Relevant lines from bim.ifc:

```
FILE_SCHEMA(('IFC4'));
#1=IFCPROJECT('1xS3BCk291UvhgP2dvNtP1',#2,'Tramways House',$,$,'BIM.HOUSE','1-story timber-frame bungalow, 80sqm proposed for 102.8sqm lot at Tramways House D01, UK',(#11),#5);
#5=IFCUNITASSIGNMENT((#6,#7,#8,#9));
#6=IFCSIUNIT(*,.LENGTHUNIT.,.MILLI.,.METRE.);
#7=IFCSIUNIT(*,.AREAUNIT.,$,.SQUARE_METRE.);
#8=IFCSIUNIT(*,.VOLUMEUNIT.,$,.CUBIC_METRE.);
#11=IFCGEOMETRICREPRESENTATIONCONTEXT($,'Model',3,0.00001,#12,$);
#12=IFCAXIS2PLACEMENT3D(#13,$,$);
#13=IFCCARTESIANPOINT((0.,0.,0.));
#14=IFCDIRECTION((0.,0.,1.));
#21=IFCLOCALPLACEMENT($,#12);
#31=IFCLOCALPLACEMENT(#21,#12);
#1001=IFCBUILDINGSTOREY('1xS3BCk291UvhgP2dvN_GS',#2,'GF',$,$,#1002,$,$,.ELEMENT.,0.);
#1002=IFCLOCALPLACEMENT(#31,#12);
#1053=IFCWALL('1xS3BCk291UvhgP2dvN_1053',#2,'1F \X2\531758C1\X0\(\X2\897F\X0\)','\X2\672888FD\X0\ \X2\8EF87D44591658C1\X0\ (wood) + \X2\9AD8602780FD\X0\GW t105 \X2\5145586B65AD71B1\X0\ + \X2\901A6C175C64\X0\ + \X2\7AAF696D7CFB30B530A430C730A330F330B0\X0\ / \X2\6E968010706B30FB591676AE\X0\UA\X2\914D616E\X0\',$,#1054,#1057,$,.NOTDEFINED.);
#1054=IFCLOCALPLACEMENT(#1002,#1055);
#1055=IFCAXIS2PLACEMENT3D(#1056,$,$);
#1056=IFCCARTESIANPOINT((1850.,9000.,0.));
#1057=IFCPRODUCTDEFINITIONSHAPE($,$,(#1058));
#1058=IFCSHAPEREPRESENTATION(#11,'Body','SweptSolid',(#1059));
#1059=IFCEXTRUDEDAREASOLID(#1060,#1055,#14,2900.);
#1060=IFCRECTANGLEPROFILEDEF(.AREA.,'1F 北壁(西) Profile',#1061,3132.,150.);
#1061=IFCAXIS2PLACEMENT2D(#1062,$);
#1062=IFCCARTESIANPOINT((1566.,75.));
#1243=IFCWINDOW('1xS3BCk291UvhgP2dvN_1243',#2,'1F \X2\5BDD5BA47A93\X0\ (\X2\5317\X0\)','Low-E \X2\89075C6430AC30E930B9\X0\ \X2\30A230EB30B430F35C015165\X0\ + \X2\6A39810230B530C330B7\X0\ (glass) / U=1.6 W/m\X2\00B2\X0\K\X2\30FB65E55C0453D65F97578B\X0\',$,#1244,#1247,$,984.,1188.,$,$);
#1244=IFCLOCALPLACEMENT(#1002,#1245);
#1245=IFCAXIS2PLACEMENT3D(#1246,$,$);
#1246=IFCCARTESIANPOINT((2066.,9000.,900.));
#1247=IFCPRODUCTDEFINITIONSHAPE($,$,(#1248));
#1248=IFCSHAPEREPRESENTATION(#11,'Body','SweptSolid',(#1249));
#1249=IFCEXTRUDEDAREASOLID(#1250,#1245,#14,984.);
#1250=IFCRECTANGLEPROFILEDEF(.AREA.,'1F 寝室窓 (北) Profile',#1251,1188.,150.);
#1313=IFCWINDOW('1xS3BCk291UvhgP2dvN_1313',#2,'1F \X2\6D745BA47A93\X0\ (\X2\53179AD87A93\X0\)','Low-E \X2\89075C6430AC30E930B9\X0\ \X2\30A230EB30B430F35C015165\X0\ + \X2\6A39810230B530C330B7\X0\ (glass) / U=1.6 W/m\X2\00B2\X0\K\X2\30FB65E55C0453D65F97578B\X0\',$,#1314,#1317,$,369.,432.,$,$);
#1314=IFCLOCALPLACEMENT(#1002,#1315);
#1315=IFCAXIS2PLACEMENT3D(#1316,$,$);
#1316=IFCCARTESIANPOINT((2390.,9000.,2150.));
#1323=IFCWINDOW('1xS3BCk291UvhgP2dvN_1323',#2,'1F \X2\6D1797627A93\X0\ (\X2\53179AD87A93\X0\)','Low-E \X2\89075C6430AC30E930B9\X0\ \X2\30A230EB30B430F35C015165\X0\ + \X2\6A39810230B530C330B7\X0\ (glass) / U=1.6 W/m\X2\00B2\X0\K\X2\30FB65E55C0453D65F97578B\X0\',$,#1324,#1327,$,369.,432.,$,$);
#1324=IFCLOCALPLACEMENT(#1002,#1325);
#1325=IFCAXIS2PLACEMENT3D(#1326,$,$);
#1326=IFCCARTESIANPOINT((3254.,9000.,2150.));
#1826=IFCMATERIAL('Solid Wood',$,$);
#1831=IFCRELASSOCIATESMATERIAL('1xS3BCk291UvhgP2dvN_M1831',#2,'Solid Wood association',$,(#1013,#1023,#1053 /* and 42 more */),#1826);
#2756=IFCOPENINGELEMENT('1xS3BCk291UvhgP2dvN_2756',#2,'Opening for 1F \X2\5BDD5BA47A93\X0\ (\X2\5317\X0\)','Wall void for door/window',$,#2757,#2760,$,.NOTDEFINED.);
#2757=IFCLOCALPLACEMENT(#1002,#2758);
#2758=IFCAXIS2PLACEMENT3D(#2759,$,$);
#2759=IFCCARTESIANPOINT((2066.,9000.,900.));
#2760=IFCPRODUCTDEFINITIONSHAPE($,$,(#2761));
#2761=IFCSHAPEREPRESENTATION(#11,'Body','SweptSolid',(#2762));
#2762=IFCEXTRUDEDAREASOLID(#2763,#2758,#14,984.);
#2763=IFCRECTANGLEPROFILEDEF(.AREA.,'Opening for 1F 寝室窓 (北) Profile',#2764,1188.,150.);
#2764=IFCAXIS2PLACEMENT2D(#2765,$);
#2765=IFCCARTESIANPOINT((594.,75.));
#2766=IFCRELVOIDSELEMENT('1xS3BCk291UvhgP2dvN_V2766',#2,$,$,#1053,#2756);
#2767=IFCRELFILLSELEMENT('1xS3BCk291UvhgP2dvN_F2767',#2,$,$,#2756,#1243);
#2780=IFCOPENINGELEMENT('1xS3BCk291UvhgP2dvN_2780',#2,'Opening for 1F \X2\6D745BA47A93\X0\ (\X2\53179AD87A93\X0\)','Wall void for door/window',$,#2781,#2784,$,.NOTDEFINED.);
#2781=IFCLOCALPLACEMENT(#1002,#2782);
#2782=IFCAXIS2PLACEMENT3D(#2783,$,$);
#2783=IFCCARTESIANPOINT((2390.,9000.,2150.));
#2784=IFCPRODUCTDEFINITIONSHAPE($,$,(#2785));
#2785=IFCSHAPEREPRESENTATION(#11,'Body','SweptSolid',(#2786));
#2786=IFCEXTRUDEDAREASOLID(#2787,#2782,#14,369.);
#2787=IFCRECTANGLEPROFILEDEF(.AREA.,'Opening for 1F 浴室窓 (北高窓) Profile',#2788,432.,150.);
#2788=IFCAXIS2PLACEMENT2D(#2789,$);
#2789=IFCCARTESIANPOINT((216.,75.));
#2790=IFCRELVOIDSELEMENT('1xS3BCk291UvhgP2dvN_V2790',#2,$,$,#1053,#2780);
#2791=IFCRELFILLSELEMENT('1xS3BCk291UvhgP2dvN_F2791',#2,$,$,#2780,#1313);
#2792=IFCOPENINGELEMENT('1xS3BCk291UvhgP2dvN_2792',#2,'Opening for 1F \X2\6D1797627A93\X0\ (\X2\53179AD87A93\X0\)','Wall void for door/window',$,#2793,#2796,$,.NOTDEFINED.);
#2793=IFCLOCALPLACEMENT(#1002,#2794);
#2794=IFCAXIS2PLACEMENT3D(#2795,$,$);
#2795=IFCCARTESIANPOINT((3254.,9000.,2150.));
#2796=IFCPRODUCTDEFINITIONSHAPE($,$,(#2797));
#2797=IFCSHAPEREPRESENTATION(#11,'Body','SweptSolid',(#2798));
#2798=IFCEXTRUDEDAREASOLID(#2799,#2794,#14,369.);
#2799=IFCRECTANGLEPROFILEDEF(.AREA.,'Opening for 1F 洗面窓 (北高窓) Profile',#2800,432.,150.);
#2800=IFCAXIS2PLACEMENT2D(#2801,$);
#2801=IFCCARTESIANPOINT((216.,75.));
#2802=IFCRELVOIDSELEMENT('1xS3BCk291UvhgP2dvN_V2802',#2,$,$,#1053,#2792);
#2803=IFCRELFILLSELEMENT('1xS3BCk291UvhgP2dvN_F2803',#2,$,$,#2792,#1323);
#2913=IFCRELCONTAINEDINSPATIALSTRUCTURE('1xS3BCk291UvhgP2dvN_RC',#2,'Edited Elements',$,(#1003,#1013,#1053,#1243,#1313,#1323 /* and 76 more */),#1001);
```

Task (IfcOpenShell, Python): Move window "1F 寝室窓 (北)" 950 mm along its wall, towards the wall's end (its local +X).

```python
import ifcopenshell
import ifcopenshell.api.geometry
import ifcopenshell.util.placement

model = ifcopenshell.open("bim.ifc")

window = model.by_guid("1xS3BCk291UvhgP2dvN_1243")
opening = window.FillsVoids[0].RelatingOpeningElement
wall = opening.VoidsElements[0].RelatingBuildingElement

wall_matrix = ifcopenshell.util.placement.get_local_placement(wall.ObjectPlacement)
shift = wall_matrix[:3, 0] * 950.0
before = ifcopenshell.util.placement.get_local_placement(window.ObjectPlacement)[:3, 3].copy()

# The window is not placed relative to its opening, so move both.
for product in (opening, window):
    matrix = ifcopenshell.util.placement.get_local_placement(product.ObjectPlacement)
    matrix[:3, 3] += shift
    ifcopenshell.api.geometry.edit_object_placement(model, product=product, matrix=matrix, is_si=False)

after = ifcopenshell.util.placement.get_local_placement(window.ObjectPlacement)[:3, 3]
print("window moved by", (after - before).round(3) + 0.0)

model.write("bim_updated.ifc")
```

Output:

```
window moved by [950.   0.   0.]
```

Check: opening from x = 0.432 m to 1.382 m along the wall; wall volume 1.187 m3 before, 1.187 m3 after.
